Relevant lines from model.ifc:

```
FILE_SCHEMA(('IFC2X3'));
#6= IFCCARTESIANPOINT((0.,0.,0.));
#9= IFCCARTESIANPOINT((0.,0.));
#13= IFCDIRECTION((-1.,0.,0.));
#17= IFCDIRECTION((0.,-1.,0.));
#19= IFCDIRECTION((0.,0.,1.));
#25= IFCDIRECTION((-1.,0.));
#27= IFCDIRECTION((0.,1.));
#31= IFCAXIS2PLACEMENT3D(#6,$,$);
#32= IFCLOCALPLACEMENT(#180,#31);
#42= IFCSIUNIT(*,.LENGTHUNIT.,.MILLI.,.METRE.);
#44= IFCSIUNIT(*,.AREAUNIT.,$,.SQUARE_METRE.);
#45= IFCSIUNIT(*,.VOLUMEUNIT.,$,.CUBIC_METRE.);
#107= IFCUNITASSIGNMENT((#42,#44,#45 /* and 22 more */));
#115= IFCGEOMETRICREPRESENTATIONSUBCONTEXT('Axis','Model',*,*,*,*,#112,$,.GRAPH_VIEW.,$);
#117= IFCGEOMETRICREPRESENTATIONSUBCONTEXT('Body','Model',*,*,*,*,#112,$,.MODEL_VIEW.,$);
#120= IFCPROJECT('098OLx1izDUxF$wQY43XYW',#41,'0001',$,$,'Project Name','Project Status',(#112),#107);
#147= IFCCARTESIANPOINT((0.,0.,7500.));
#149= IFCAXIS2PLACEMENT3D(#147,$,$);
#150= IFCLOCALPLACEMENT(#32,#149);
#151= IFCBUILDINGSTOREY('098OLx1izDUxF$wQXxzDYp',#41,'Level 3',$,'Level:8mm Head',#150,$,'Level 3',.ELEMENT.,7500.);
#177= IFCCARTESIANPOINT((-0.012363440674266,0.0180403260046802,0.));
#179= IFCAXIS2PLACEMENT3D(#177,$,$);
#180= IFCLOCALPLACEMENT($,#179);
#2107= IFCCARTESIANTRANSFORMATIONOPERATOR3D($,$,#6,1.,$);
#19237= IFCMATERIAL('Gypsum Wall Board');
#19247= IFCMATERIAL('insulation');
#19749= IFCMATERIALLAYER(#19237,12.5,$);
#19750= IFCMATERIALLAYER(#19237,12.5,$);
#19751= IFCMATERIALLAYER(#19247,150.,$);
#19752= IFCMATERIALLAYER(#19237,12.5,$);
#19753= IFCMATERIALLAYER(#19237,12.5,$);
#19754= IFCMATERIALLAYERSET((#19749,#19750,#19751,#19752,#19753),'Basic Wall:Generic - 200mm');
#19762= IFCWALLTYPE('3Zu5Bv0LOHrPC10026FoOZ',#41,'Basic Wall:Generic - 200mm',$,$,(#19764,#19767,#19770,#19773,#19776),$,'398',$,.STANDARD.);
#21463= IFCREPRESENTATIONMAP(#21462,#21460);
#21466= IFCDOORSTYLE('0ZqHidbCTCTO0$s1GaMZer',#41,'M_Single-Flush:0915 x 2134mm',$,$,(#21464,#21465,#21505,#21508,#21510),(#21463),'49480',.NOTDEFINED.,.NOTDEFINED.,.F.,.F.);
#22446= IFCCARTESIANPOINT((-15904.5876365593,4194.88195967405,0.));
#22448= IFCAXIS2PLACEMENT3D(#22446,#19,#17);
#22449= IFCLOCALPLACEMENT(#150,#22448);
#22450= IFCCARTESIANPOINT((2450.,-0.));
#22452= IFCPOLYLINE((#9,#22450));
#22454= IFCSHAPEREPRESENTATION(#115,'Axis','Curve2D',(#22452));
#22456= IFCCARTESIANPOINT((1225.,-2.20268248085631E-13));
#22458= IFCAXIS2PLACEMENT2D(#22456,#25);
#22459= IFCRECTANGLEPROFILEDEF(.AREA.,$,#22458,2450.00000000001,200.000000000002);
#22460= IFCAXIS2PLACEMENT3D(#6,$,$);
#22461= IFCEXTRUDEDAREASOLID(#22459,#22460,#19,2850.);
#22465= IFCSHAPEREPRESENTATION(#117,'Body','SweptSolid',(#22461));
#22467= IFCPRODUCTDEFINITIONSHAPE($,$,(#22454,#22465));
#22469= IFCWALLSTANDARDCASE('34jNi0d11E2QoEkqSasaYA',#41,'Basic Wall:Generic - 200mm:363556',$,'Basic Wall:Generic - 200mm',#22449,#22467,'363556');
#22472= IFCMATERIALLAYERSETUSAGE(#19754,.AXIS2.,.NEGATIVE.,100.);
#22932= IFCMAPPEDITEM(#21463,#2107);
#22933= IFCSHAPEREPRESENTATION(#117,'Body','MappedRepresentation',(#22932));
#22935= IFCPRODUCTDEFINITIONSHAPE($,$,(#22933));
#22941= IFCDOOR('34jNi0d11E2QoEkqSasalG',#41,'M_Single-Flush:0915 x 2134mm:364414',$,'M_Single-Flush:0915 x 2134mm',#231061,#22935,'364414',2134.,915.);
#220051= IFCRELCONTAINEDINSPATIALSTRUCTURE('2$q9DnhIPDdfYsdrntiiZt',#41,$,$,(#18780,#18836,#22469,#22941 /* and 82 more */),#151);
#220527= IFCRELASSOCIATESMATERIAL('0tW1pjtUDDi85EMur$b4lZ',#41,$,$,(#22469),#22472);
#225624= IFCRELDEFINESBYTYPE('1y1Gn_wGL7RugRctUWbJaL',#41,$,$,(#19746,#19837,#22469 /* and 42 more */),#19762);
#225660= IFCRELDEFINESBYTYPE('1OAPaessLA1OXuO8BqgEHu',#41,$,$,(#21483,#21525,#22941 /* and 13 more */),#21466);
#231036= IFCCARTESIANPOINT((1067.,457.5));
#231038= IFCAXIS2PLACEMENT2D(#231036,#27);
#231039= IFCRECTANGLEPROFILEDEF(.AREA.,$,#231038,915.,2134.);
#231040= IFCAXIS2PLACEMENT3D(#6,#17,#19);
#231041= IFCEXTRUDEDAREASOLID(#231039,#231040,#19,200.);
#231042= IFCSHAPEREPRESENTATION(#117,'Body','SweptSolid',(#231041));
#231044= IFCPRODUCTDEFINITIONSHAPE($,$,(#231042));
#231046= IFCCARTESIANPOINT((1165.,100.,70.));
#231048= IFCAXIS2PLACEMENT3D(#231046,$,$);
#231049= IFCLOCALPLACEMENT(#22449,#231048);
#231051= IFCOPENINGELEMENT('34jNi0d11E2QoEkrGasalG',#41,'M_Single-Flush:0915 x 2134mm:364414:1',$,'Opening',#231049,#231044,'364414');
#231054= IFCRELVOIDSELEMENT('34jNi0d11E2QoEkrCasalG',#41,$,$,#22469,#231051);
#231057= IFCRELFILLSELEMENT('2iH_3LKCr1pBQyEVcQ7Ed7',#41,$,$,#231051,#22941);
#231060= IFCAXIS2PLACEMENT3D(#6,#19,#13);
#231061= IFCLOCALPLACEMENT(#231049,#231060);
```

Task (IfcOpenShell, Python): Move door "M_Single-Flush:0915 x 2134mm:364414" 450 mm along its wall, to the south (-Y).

```python
import ifcopenshell
import ifcopenshell.api.geometry
import ifcopenshell.util.placement

model = ifcopenshell.open("model.ifc")

door = model.by_guid("34jNi0d11E2QoEkqSasalG")
opening = door.FillsVoids[0].RelatingOpeningElement
wall = opening.VoidsElements[0].RelatingBuildingElement

wall_matrix = ifcopenshell.util.placement.get_local_placement(wall.ObjectPlacement)
shift = wall_matrix[:3, 0] * 450.0
before = ifcopenshell.util.placement.get_local_placement(door.ObjectPlacement)[:3, 3].copy()

# The door is placed relative to its opening, so it follows when the opening moves.
matrix = ifcopenshell.util.placement.get_local_placement(opening.ObjectPlacement)
matrix[:3, 3] += shift
ifcopenshell.api.geometry.edit_object_placement(
    model, product=opening, matrix=matrix, is_si=False, should_transform_children=True
)

after = ifcopenshell.util.placement.get_local_placement(door.ObjectPlacement)[:3, 3]
print("door moved by", (after - before).round(3) + 0.0)

model.write("model-out.ifc")
```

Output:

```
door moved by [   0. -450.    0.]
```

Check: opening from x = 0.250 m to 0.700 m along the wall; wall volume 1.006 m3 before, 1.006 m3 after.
